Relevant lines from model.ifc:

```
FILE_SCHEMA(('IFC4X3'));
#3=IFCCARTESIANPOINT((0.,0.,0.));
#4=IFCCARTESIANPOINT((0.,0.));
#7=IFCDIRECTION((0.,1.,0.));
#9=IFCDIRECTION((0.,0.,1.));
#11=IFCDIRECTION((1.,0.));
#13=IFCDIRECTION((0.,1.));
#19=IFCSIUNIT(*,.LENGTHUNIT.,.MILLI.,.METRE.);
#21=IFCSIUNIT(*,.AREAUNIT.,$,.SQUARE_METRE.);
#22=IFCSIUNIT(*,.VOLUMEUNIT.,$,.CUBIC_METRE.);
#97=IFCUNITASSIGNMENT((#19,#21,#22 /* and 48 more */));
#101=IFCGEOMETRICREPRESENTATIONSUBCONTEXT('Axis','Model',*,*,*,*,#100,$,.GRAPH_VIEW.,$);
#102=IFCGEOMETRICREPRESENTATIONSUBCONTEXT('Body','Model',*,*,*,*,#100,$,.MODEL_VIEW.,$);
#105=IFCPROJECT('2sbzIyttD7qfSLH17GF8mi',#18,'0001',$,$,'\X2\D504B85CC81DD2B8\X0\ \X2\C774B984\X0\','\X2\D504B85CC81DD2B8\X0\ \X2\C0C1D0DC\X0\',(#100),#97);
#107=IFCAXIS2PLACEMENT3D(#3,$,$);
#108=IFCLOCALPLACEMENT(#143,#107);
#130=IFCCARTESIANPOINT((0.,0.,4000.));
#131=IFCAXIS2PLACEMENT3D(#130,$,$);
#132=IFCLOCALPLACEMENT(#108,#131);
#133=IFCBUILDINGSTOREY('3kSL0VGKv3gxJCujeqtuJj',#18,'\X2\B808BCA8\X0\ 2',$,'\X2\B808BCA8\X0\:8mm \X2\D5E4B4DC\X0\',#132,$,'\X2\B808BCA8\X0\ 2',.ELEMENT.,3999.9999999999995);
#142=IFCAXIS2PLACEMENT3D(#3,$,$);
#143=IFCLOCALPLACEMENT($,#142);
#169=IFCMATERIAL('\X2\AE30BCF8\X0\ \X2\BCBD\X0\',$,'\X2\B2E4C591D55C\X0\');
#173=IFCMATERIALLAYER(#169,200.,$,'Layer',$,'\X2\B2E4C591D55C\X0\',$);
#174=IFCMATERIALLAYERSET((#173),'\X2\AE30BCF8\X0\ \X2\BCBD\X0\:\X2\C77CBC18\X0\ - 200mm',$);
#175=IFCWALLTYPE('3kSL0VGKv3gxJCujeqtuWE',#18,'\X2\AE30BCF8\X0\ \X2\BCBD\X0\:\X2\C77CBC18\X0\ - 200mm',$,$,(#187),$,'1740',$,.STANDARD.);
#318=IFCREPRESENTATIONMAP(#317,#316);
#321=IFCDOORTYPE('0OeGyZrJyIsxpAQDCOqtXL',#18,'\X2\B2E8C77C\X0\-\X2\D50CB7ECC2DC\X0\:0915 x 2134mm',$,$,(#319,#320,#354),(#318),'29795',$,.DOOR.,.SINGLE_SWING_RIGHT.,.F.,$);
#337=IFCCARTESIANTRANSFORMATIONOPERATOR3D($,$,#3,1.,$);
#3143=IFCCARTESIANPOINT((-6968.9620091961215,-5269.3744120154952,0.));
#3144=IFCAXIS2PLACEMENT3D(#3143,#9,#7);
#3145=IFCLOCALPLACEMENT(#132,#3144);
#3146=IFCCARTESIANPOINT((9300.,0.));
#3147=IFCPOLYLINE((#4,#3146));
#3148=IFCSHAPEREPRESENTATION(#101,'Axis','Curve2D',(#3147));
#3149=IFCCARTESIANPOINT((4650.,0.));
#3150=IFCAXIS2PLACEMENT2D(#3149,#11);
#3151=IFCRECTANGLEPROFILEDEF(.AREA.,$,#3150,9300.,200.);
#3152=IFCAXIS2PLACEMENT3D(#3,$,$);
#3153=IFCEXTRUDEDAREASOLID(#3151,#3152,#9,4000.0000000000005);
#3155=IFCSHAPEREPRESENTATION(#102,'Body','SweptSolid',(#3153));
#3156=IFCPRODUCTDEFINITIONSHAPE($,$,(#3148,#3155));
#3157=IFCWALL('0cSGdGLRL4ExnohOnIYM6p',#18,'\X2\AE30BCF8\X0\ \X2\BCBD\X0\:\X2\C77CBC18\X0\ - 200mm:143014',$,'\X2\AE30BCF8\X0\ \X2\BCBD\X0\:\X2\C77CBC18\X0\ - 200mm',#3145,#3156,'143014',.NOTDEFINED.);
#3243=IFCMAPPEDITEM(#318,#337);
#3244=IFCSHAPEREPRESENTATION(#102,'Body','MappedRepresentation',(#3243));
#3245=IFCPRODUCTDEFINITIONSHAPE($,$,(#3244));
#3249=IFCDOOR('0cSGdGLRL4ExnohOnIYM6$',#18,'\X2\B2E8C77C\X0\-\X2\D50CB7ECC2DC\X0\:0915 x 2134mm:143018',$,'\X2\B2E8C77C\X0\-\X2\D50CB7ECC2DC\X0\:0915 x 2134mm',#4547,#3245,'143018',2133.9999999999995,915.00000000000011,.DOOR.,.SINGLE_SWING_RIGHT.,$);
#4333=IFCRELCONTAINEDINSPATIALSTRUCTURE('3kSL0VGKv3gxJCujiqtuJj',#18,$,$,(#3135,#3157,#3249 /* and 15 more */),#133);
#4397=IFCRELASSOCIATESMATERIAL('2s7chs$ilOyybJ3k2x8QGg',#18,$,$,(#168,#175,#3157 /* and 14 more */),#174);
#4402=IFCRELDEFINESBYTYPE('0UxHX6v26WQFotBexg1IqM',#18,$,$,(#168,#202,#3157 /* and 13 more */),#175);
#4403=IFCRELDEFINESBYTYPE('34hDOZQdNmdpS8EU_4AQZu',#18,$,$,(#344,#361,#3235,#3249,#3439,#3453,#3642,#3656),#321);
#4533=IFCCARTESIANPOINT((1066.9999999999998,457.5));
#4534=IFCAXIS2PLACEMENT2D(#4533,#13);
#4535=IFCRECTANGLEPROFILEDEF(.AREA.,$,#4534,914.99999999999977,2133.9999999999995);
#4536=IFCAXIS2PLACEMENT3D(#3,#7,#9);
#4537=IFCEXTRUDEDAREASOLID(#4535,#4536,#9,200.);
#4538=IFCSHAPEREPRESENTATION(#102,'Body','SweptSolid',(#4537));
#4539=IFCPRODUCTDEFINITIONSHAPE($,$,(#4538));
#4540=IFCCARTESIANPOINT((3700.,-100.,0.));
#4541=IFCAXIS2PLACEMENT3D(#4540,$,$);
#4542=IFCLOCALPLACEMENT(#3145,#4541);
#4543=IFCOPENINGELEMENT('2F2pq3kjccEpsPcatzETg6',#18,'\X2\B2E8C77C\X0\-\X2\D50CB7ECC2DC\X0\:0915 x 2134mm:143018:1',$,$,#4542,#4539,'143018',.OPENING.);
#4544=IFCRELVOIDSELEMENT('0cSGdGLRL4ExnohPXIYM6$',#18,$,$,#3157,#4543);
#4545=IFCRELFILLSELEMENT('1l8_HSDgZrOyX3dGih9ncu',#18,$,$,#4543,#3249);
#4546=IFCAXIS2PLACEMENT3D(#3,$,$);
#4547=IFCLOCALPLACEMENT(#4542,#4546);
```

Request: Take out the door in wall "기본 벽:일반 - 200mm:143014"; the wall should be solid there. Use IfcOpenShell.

```python
import ifcopenshell
import ifcopenshell.api.feature
import ifcopenshell.api.root
import ifcopenshell.geom
import ifcopenshell.util.shape

model = ifcopenshell.open("model.ifc")
settings = ifcopenshell.geom.settings()


def volume(element):
    """Net volume in cubic metres, openings subtracted."""
    shape = ifcopenshell.geom.create_shape(settings, element)
    return ifcopenshell.util.shape.get_volume(shape.geometry)


door = model.by_guid("0cSGdGLRL4ExnohOnIYM6$")
opening = door.FillsVoids[0].RelatingOpeningElement
wall = opening.VoidsElements[0].RelatingBuildingElement
before = volume(wall)

ifcopenshell.api.root.remove_product(model, product=door)
ifcopenshell.api.feature.remove_feature(model, feature=opening)

after = volume(wall)

print(f"wall volume {before:.3f} -> {after:.3f} m3")

model.write("model_v2.ifc")
```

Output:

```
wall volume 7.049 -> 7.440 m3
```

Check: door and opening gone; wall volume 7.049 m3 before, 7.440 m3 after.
